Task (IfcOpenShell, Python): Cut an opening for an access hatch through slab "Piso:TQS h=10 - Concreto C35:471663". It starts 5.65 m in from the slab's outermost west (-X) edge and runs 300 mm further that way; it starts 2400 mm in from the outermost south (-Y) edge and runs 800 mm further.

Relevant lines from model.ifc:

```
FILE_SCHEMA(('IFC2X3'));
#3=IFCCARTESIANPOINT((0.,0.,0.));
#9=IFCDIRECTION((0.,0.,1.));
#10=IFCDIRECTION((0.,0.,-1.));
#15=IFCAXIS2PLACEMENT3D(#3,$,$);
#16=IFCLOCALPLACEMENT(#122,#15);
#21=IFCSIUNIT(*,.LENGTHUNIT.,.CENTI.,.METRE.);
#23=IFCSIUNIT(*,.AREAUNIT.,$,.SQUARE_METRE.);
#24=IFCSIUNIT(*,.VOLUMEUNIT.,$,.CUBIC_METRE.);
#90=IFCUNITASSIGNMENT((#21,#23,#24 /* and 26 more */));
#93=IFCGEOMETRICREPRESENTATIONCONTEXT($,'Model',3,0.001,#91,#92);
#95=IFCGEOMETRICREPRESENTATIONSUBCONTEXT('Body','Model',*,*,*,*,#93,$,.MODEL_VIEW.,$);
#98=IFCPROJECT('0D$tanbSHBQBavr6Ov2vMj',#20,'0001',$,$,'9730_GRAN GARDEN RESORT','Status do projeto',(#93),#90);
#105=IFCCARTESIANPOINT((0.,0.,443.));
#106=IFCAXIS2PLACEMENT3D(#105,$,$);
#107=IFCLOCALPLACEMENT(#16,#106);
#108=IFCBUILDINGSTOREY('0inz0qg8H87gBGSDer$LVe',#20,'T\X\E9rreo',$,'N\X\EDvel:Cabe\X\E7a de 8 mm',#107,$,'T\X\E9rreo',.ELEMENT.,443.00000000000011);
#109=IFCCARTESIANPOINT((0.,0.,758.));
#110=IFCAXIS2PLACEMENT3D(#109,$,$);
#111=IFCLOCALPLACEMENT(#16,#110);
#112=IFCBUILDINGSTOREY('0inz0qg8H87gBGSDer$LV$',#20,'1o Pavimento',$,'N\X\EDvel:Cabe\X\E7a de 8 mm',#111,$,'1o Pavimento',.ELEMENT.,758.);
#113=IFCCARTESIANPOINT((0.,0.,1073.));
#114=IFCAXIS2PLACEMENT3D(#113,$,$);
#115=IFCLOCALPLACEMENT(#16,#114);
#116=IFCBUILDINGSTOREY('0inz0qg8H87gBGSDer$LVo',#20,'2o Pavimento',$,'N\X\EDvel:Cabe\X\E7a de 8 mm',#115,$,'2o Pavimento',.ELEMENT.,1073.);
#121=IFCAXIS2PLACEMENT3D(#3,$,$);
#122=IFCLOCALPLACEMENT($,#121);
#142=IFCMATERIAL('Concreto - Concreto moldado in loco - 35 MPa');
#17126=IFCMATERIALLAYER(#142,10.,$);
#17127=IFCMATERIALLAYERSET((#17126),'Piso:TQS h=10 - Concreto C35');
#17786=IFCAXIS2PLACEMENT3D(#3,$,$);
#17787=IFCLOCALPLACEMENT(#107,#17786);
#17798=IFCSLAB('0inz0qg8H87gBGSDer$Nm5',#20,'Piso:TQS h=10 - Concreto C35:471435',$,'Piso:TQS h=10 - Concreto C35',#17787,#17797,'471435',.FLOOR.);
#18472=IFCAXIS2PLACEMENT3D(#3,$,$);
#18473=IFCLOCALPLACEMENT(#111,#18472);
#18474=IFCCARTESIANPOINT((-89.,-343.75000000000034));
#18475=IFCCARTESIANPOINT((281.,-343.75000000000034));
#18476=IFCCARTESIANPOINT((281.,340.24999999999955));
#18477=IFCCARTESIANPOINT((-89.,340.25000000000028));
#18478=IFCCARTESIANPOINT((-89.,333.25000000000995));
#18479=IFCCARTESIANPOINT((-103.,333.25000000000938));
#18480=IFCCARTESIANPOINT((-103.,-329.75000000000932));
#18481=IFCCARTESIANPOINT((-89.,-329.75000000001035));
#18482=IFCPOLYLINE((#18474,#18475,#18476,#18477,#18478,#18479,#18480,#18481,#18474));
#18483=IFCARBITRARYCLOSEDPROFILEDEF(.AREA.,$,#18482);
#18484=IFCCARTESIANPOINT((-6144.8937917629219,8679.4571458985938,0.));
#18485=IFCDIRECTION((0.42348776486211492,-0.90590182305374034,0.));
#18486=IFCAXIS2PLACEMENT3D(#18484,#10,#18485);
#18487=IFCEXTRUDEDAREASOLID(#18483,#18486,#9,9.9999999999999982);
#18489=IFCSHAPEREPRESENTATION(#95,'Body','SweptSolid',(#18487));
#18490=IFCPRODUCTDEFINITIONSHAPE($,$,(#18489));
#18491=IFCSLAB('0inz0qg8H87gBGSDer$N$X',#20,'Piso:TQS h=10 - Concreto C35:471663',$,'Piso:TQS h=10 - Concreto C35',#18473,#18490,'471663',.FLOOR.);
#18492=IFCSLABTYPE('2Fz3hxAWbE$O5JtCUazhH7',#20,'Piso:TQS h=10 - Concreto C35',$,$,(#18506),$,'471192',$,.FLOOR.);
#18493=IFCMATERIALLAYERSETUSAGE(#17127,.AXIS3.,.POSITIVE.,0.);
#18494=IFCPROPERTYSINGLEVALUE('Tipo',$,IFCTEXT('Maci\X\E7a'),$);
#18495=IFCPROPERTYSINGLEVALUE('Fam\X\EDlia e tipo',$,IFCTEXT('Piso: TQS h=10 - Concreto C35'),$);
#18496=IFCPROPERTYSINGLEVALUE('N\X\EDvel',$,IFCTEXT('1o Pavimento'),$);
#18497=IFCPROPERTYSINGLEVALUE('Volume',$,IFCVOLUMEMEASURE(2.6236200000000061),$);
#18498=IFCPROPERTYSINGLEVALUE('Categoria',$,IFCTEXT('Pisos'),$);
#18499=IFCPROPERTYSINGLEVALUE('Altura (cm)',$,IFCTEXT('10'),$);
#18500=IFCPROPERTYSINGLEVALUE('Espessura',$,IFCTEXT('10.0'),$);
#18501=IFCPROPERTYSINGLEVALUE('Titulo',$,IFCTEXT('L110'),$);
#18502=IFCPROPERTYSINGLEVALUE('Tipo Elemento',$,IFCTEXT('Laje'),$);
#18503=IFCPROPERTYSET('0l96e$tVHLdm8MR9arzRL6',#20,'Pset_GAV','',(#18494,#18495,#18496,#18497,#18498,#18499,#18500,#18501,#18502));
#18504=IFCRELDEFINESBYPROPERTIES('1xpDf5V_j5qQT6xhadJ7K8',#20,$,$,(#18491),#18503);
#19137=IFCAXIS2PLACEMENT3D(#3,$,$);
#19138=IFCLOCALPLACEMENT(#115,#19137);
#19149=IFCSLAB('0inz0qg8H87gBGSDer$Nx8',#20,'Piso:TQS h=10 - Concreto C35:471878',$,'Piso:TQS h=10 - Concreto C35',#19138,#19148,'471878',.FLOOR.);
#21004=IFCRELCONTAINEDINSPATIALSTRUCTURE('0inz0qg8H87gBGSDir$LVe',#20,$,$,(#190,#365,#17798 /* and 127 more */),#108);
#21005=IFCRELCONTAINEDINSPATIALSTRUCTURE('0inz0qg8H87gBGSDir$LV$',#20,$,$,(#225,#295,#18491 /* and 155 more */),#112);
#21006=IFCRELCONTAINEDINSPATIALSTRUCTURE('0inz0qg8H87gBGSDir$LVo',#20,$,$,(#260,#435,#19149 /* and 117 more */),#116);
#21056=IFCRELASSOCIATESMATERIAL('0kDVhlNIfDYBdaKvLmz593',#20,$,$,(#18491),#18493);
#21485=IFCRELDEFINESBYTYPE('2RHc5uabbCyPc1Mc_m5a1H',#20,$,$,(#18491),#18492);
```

```python
import numpy as np
import ifcopenshell
import ifcopenshell.api.feature
import ifcopenshell.api.geometry
import ifcopenshell.api.pset
import ifcopenshell.api.root
import ifcopenshell.geom
import ifcopenshell.util.element
import ifcopenshell.util.placement
import ifcopenshell.util.representation
import ifcopenshell.util.shape
import ifcopenshell.util.unit

model = ifcopenshell.open("model.ifc")
unit_scale = ifcopenshell.util.unit.calculate_unit_scale(model)
volume_scale = ifcopenshell.util.unit.calculate_unit_scale(model, "VOLUMEUNIT")
settings = ifcopenshell.geom.settings()


def volume(element):
    """Net volume in cubic metres, openings subtracted."""
    shape = ifcopenshell.geom.create_shape(settings, element)
    return ifcopenshell.util.shape.get_volume(shape.geometry)


slab = model.by_guid("0inz0qg8H87gBGSDer$N$X")
before = volume(slab)

# Extent in the slab's own axes, in metres. The edges named are its -X and -Y sides.
slab_shape = ifcopenshell.geom.create_shape(settings, slab)
vertices = ifcopenshell.util.shape.get_vertices(slab_shape.geometry)
x_min, y_min, bottom = vertices.min(axis=0)
top = vertices[:, 2].max()

opening = ifcopenshell.api.root.create_entity(model, ifc_class="IfcOpeningElement", name="Access hatch opening")
context = ifcopenshell.util.representation.get_context(model, "Model", "Body", "MODEL_VIEW")
width, depth = 0.3, 0.8
outline = [(0.0, 0.0), (width, 0.0), (width, depth), (0.0, depth), (0.0, 0.0)]
# Overshoot both faces by 50 mm so the cut is clean.
shape = ifcopenshell.api.geometry.add_slab_representation(
    model, context=context, depth=top - bottom + 0.1, polyline=outline
)
ifcopenshell.api.geometry.assign_representation(model, product=opening, representation=shape)

matrix = ifcopenshell.util.placement.get_local_placement(slab.ObjectPlacement)
matrix[:, 3] = matrix @ np.append(np.array([x_min + 5.65, y_min + 2.4, bottom - 0.05]) / unit_scale, 1.0)
ifcopenshell.api.geometry.edit_object_placement(model, product=opening, matrix=matrix, is_si=False)
ifcopenshell.api.feature.add_feature(model, feature=opening, element=slab)

after = volume(slab)

# Update the slab's stored quantities.
pset = model.by_id(ifcopenshell.util.element.get_pset(slab, "Pset_GAV", should_inherit=False)["id"])
ifcopenshell.api.pset.edit_pset(model, pset=pset, properties={
    "Volume": model.create_entity("IfcVolumeMeasure", after / volume_scale),
})

print(f"slab volume {before:.3f} -> {after:.3f} m3")

model.write("model_updated.ifc")
```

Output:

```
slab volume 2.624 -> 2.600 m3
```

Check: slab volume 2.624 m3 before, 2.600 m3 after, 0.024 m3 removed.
